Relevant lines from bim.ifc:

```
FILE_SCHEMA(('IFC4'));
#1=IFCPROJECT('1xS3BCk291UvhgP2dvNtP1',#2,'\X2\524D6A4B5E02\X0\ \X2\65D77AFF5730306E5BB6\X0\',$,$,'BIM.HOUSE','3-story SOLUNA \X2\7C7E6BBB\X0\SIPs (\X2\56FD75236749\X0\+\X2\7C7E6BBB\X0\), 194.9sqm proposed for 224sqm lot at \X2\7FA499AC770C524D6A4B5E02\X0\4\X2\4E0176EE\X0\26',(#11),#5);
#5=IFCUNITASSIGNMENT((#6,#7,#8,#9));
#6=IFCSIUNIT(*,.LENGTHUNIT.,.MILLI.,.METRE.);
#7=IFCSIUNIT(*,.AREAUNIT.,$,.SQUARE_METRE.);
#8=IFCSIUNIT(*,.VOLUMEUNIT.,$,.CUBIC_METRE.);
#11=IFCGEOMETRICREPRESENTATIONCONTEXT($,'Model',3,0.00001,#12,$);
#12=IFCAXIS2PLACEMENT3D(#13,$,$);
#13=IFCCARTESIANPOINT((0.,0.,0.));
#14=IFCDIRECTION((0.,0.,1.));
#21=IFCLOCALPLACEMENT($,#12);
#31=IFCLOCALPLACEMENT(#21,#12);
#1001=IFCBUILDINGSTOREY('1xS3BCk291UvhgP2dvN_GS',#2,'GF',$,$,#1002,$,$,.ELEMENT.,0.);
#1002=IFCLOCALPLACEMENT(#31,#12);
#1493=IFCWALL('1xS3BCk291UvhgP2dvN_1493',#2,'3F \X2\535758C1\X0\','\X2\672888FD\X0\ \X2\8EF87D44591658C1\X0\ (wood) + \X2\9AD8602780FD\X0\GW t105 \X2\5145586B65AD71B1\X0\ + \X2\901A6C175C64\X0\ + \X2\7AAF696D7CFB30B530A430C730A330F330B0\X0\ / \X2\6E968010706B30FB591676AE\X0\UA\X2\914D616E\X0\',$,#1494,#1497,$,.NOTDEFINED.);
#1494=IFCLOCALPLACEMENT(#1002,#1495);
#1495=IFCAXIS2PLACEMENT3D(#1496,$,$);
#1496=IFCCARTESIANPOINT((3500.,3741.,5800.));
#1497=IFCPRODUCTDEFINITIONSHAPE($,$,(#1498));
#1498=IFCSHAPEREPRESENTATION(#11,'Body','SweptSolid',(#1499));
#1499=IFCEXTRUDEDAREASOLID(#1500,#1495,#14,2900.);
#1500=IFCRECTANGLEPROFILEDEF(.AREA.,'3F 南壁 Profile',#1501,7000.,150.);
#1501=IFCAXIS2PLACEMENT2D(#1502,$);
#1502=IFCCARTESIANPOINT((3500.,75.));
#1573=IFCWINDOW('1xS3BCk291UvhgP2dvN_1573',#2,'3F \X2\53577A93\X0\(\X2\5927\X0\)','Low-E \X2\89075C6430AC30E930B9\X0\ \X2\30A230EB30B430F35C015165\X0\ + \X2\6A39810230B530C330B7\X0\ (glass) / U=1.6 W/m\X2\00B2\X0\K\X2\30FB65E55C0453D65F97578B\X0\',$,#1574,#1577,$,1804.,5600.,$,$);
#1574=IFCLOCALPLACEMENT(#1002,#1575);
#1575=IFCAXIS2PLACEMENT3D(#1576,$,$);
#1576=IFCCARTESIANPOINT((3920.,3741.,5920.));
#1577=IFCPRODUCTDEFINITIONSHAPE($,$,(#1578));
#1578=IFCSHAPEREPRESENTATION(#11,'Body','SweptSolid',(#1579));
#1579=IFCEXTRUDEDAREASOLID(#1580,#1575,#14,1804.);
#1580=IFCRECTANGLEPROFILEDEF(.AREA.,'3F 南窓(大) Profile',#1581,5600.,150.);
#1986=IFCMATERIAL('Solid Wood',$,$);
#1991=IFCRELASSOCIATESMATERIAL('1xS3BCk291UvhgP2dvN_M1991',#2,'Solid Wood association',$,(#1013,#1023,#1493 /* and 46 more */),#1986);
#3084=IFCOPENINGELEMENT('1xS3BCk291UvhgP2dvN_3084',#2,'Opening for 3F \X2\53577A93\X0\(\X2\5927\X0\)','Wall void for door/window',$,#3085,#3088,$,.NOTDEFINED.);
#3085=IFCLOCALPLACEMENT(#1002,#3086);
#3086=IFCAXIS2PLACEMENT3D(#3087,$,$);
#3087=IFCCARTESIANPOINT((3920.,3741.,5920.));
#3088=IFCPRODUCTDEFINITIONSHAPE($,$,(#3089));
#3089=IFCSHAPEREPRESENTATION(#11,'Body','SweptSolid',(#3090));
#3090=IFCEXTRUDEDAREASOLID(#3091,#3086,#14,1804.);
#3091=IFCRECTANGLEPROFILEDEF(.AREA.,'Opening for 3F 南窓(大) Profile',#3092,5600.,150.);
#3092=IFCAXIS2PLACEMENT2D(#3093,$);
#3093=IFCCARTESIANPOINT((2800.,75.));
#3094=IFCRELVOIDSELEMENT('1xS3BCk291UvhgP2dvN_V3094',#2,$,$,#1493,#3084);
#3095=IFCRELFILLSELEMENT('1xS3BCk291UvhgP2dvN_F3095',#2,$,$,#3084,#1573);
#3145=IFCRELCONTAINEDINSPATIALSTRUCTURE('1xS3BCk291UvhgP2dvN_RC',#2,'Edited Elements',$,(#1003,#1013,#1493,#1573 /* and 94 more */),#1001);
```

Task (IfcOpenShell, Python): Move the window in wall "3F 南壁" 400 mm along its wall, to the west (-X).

```python
import ifcopenshell
import ifcopenshell.api.geometry
import ifcopenshell.util.placement
import ifcopenshell.util.unit

model = ifcopenshell.open("bim.ifc")
unit_scale = ifcopenshell.util.unit.calculate_unit_scale(model)

window = model.by_guid("1xS3BCk291UvhgP2dvN_1573")
opening = window.FillsVoids[0].RelatingOpeningElement
wall = opening.VoidsElements[0].RelatingBuildingElement

wall_matrix = ifcopenshell.util.placement.get_local_placement(wall.ObjectPlacement)
shift = wall_matrix[:3, 0] * -0.4 / unit_scale
before = ifcopenshell.util.placement.get_local_placement(window.ObjectPlacement)[:3, 3].copy()

# The window is not placed relative to its opening, so move both.
for product in (opening, window):
    matrix = ifcopenshell.util.placement.get_local_placement(product.ObjectPlacement)
    matrix[:3, 3] += shift
    ifcopenshell.api.geometry.edit_object_placement(model, product=product, matrix=matrix, is_si=False)

after = ifcopenshell.util.placement.get_local_placement(window.ObjectPlacement)[:3, 3]
print("window moved by", (after - before).round(3) + 0.0)

model.write("bim_edited.ifc")
```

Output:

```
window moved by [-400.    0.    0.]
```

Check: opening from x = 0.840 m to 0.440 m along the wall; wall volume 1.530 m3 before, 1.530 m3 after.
